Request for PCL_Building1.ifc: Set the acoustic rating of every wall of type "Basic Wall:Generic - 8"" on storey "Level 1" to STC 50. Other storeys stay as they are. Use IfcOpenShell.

First a look at what the model holds.

```python
import ifcopenshell
import ifcopenshell.util.element

model = ifcopenshell.open("PCL_Building1.ifc")
print(model.schema)
storey = next(s for s in model.by_type("IfcBuildingStorey") if s.Name == "Level 1")
walls = [e for e in ifcopenshell.util.element.get_decomposition(storey) if e.is_a("IfcWall")]
seen = {}
for e in walls:
    element_type = ifcopenshell.util.element.get_type(e)
    key = (element_type.Name if element_type != e and element_type else None, ifcopenshell.util.element.get_pset(e, "Pset_WallCommon", "AcousticRating"))
    seen[key] = seen.get(key, 0) + 1
for (name, value), count in sorted(seen.items(), key=str):
    print(count, "x", name, "|", value)
```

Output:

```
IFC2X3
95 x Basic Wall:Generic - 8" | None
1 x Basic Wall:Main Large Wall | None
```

```python
import ifcopenshell
import ifcopenshell.api.pset
import ifcopenshell.util.element

model = ifcopenshell.open("PCL_Building1.ifc")

storey = next(s for s in model.by_type("IfcBuildingStorey") if s.Name == "Level 1")
walls = [e for e in ifcopenshell.util.element.get_decomposition(storey) if e.is_a("IfcWall")]

count = 0
for e in walls:
    element_type = ifcopenshell.util.element.get_type(e)
    if element_type in (None, e) or element_type.Name != 'Basic Wall:Generic - 8"':
        continue
    # add_pset returns the element's existing set when there is one.
    pset = ifcopenshell.api.pset.add_pset(model, product=e, name="Pset_WallCommon")
    ifcopenshell.api.pset.edit_pset(model, pset=pset, properties={"AcousticRating": "STC 50"})
    count += 1

print(count, "walls updated")

model.write("PCL_Building1_rev.ifc")
```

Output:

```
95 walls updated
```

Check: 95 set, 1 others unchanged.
